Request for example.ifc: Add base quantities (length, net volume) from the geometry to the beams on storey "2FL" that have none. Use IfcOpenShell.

First a look at what the model holds.

```python
import ifcopenshell
import ifcopenshell.util.element
import ifcopenshell.util.unit

model = ifcopenshell.open("example.ifc")
print(model.schema)
for unit_type in ("LENGTHUNIT", "AREAUNIT", "VOLUMEUNIT"):
    print(unit_type, ifcopenshell.util.unit.calculate_unit_scale(model, unit_type))
storey = next(s for s in model.by_type("IfcBuildingStorey") if s.Name == "2FL")
beams = [e for e in ifcopenshell.util.element.get_decomposition(storey) if e.is_a("IfcBeam")]
for e in sorted(beams, key=lambda e: e.id()):
    print(e.id(), e.is_a(), e.Name, list(ifcopenshell.util.element.get_psets(e, qtos_only=True)), sep=" | ")
```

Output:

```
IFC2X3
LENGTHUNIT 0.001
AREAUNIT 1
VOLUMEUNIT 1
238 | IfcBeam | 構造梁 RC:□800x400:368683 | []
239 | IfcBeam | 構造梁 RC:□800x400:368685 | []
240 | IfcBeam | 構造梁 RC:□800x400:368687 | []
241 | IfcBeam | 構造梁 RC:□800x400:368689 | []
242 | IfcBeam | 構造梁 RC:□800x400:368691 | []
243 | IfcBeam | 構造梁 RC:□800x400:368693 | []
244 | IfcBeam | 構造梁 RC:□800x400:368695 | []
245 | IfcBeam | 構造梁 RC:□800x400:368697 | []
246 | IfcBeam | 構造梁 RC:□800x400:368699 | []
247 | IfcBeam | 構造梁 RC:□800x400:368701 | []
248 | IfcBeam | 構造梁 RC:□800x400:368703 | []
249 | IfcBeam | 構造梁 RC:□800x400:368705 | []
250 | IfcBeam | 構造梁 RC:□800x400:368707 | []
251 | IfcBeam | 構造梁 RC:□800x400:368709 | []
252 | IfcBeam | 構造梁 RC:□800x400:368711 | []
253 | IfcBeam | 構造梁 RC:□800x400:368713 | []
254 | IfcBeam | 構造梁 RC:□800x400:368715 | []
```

```python
import ifcopenshell
import ifcopenshell.api.pset
import ifcopenshell.geom
import ifcopenshell.util.element
import ifcopenshell.util.shape
import ifcopenshell.util.unit

model = ifcopenshell.open("example.ifc")
unit_scale = ifcopenshell.util.unit.calculate_unit_scale(model)
volume_scale = ifcopenshell.util.unit.calculate_unit_scale(model, "VOLUMEUNIT")
settings = ifcopenshell.geom.settings()

storey = next(s for s in model.by_type("IfcBuildingStorey") if s.Name == "2FL")
beams = [e for e in ifcopenshell.util.element.get_decomposition(storey) if e.is_a("IfcBeam")]

for e in sorted(beams, key=lambda e: e.id()):
    if ifcopenshell.util.element.get_psets(e, qtos_only=True, should_inherit=False):
        continue
    # Geometry comes back in metres, in the element's own axes.
    shape = ifcopenshell.geom.create_shape(settings, e)
    values = {
        "Length": ifcopenshell.util.shape.get_max_xyz(shape.geometry) / unit_scale,
        "NetVolume": ifcopenshell.util.shape.get_volume(shape.geometry) / volume_scale,
    }
    qto = ifcopenshell.api.pset.add_qto(model, product=e, name="BaseQuantities")
    ifcopenshell.api.pset.edit_qto(model, qto=qto, properties=values)
    print(e.id(), {k: round(v, 3) for k, v in values.items()})

model.write("example-out.ifc")
```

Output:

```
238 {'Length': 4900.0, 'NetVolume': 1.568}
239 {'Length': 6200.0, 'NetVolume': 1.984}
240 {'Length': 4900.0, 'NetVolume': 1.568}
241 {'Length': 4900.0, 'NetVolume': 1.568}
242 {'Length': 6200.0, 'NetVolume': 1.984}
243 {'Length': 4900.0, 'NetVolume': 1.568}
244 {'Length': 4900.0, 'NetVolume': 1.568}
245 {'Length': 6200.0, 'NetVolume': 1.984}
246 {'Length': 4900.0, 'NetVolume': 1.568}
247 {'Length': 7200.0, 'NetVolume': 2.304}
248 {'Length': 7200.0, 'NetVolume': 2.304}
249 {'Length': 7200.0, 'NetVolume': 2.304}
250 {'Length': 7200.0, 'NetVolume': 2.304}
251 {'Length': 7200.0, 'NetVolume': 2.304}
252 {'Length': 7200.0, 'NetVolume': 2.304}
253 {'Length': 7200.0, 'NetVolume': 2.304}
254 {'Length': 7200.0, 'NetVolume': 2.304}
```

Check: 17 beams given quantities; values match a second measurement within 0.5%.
